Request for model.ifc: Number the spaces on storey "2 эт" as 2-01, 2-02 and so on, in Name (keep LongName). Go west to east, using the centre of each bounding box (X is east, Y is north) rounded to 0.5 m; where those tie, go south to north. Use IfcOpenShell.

First a look at what the model holds.

```python
import ifcopenshell
import ifcopenshell.util.element
import ifcopenshell.util.placement

model = ifcopenshell.open("model.ifc")
print(model.schema)
storey = next(s for s in model.by_type("IfcBuildingStorey") if s.Name == "2 эт")
spaces = [e for e in ifcopenshell.util.element.get_decomposition(storey) if e.is_a("IfcSpace")]
for e in sorted(spaces, key=lambda e: e.id()):
    origin = ifcopenshell.util.placement.get_local_placement(e.ObjectPlacement)[:3, 3]
    print(e.id(), e.Name, e.LongName, origin.round(2) + 0.0, sep=" | ")
```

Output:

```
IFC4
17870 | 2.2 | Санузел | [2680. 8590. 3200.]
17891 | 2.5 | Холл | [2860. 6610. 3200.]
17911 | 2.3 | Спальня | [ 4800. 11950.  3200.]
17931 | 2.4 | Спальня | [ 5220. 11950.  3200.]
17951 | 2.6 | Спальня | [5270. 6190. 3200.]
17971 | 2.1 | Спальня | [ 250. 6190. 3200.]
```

```python
import ifcopenshell
import ifcopenshell.geom
import ifcopenshell.util.element
import ifcopenshell.util.shape

model = ifcopenshell.open("model.ifc")
settings = ifcopenshell.geom.settings()
settings.set("use-world-coords", True)


def centre(element):
    shape = ifcopenshell.geom.create_shape(settings, element)
    return ifcopenshell.util.shape.get_bbox_centroid(shape.geometry)


storey = next(s for s in model.by_type("IfcBuildingStorey") if s.Name == "2 эт")
spaces = [e for e in ifcopenshell.util.element.get_decomposition(storey) if e.is_a("IfcSpace")]

# Insertion points can sit at a corner or the storey origin, so sort by the geometry (in metres).
centres = {e: centre(e) for e in spaces}
spaces.sort(key=lambda e: (round(centres[e][0] / 0.5), centres[e][1]))

for i, e in enumerate(spaces, start=1):
    number = f"2-{i:02d}"
    e.Name = number
    print(e.id(), number)

model.write("model_updated.ifc")
```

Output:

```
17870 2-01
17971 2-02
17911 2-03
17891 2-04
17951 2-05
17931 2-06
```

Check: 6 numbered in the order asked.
